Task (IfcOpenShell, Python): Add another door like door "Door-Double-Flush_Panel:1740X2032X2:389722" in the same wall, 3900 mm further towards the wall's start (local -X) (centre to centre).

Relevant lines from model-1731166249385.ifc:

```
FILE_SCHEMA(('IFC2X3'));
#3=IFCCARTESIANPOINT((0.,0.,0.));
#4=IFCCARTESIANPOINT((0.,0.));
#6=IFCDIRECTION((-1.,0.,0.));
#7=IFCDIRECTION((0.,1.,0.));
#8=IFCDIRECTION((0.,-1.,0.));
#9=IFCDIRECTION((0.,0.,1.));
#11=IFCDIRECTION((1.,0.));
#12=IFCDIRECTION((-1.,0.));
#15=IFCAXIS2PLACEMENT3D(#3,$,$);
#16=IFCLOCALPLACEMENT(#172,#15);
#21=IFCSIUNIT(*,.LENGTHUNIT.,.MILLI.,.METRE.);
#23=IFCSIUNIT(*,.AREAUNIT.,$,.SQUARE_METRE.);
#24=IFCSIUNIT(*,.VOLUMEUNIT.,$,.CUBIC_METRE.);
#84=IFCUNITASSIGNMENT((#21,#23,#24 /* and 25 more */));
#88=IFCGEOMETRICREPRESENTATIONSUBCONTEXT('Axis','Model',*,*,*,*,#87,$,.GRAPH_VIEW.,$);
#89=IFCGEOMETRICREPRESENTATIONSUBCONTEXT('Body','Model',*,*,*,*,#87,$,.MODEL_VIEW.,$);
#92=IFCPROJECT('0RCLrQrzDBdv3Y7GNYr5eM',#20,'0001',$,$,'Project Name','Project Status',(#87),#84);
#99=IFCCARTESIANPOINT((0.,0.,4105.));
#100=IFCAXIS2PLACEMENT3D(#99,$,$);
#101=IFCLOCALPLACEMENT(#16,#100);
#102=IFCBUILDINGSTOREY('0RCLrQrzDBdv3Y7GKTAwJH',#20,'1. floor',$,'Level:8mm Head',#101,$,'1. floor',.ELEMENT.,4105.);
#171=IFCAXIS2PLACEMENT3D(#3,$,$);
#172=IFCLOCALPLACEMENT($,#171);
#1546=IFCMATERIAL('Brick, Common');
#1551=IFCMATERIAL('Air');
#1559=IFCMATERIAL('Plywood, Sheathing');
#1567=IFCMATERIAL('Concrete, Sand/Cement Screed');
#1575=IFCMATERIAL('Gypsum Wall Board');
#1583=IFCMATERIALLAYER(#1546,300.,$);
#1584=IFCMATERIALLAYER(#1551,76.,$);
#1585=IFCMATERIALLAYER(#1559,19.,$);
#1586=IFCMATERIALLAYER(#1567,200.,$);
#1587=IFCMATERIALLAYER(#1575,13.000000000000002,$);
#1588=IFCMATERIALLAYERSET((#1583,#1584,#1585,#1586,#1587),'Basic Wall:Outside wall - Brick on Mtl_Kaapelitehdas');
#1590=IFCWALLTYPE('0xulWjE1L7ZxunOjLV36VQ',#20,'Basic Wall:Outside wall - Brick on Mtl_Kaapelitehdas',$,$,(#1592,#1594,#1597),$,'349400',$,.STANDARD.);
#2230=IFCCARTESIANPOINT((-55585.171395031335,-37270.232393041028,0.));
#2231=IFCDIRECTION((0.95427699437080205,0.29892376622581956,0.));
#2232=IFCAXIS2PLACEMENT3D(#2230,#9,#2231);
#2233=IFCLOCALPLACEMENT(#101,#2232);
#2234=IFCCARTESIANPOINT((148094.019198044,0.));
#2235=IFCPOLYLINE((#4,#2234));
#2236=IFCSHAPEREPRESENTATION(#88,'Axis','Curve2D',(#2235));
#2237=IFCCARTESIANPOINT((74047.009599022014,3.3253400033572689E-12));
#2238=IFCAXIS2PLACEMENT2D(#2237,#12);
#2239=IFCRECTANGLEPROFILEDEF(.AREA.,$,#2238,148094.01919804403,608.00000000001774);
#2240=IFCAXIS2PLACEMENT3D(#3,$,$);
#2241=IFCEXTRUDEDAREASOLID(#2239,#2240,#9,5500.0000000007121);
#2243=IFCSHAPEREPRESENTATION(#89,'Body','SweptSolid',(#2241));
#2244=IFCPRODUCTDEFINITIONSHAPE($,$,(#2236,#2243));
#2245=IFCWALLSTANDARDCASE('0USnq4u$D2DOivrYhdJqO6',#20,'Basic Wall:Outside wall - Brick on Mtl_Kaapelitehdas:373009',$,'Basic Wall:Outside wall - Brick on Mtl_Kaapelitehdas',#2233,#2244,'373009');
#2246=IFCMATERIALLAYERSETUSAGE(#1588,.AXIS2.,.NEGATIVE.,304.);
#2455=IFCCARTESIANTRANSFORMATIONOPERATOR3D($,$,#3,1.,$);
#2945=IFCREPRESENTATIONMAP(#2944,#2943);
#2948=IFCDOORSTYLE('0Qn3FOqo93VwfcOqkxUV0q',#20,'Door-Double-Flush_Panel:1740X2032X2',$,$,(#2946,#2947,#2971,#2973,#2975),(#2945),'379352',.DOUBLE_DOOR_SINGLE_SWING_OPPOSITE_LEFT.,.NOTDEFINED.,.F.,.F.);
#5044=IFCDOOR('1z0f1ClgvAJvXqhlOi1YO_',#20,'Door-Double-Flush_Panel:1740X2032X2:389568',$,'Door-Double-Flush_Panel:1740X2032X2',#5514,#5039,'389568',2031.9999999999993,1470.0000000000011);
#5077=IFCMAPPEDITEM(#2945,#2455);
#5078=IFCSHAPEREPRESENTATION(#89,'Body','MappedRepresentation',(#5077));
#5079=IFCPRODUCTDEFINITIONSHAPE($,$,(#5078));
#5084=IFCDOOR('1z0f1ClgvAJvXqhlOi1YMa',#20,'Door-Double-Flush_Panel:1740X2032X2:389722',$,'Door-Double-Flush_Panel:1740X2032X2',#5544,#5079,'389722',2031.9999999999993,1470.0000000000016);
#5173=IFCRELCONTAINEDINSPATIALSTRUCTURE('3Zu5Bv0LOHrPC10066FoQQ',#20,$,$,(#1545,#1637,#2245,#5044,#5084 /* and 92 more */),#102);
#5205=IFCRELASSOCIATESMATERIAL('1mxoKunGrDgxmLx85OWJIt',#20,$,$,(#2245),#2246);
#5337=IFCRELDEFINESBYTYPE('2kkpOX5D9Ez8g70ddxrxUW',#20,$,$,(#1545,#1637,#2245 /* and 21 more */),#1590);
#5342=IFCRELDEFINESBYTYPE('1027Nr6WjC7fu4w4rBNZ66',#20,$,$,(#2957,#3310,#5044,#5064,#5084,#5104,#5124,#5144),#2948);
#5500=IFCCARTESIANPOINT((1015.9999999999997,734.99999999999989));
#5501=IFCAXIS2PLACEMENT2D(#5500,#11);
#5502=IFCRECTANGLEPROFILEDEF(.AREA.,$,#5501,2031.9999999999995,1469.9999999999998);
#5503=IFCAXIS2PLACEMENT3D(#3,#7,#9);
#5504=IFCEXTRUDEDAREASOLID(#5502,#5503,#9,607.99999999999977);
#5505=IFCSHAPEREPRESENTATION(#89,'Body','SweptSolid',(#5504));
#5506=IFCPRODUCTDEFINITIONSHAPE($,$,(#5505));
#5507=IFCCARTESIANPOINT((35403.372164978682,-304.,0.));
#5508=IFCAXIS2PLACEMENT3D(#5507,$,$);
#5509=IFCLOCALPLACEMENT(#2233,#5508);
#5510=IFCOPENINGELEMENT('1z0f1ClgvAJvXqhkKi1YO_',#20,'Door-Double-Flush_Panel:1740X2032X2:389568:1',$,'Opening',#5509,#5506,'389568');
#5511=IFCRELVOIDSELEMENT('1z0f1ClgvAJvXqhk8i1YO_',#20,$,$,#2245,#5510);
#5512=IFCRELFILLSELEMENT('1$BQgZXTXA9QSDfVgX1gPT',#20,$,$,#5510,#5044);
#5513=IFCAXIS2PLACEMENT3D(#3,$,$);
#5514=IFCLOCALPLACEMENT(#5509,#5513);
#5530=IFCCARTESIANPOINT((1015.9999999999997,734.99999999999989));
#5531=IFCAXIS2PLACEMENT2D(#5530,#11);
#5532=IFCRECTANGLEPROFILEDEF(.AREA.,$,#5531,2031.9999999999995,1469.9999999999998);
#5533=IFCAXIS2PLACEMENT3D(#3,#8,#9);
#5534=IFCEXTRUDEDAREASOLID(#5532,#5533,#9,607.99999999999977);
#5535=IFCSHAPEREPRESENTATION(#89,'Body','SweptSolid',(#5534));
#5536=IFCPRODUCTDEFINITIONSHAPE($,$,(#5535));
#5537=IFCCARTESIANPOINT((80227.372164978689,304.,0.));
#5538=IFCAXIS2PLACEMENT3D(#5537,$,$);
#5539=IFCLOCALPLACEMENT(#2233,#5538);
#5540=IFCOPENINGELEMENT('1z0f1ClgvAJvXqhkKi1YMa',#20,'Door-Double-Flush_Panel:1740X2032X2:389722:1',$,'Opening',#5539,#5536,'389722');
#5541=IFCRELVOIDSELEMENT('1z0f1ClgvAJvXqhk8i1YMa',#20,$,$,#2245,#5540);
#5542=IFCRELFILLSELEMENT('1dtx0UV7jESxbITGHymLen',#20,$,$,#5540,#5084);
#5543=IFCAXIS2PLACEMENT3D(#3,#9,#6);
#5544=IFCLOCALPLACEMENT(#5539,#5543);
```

```python
import ifcopenshell
import ifcopenshell.api.feature
import ifcopenshell.api.geometry
import ifcopenshell.api.root
import ifcopenshell.geom
import ifcopenshell.util.element
import ifcopenshell.util.placement
import ifcopenshell.util.shape

model = ifcopenshell.open("model-1731166249385.ifc")
settings = ifcopenshell.geom.settings()


def volume(element):
    """Net volume in cubic metres, openings subtracted."""
    shape = ifcopenshell.geom.create_shape(settings, element)
    return ifcopenshell.util.shape.get_volume(shape.geometry)


def reuse_history(source, copy):
    """copy_class also copies each property set's owner history, people and application; keep the originals."""
    for rel in copy.IsDefinedBy:
        if rel.is_a("IfcRelDefinesByProperties") and (history := rel.RelatingPropertyDefinition.OwnerHistory):
            rel.RelatingPropertyDefinition.OwnerHistory = source.OwnerHistory
            ifcopenshell.util.element.remove_deep2(model, history)


door = model.by_id(5084)
opening = door.FillsVoids[0].RelatingOpeningElement
wall = opening.VoidsElements[0].RelatingBuildingElement
before = volume(wall)
shift = ifcopenshell.util.placement.get_local_placement(wall.ObjectPlacement)[:3, 0] * -3900.0

# copy_class copies the void relationship, type, container and properties, but no geometry.
new_opening = ifcopenshell.api.root.copy_class(model, product=opening)
new_opening.Representation = ifcopenshell.util.element.copy_deep(
    model, opening.Representation, exclude=["IfcGeometricRepresentationContext", "IfcRepresentationMap"]
)
new_opening.Name = "Door-Double-Flush_Panel:1740X2032X2"
new_opening.Tag = None
new_door = ifcopenshell.api.root.copy_class(model, product=door)
new_door.Representation = ifcopenshell.util.element.copy_deep(
    model, door.Representation, exclude=["IfcGeometricRepresentationContext", "IfcRepresentationMap"]
)
new_door.Name = "Door-Double-Flush_Panel:1740X2032X2"
new_door.Tag = None
reuse_history(door, new_door)
fills = ifcopenshell.api.feature.add_filling(model, opening=new_opening, element=new_door)
fills.OwnerHistory = new_door.OwnerHistory  # required in IFC2X3

for old, new in ((opening, new_opening), (door, new_door)):
    matrix = ifcopenshell.util.placement.get_local_placement(old.ObjectPlacement)
    matrix[:3, 3] += shift
    ifcopenshell.api.geometry.edit_object_placement(model, product=new, matrix=matrix, is_si=False)

after = volume(wall)

print(f"wall volume {before:.3f} -> {after:.3f} m3")

model.write("model-1731166249385_edited.ifc")
```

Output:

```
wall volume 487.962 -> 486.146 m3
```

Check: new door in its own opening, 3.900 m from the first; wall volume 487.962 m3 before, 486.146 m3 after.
